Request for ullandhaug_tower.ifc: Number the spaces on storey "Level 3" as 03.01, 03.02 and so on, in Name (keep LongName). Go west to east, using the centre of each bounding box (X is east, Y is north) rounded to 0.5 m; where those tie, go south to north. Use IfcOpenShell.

First a look at what the model holds.

```python
import ifcopenshell
import ifcopenshell.util.element
import ifcopenshell.util.placement

model = ifcopenshell.open("ullandhaug_tower.ifc")
print(model.schema)
storey = next(s for s in model.by_type("IfcBuildingStorey") if s.Name == "Level 3")
spaces = [e for e in ifcopenshell.util.element.get_decomposition(storey) if e.is_a("IfcSpace")]
for e in sorted(spaces, key=lambda e: e.id()):
    origin = ifcopenshell.util.placement.get_local_placement(e.ObjectPlacement)[:3, 3]
    print(e.id(), e.Name, e.LongName, origin.round(2) + 0.0, sep=" | ")
```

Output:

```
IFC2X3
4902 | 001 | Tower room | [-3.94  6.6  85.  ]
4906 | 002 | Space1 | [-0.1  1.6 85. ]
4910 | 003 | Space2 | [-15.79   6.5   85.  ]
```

```python
import ifcopenshell
import ifcopenshell.geom
import ifcopenshell.util.element
import ifcopenshell.util.shape

model = ifcopenshell.open("ullandhaug_tower.ifc")
settings = ifcopenshell.geom.settings()
settings.set("use-world-coords", True)


def centre(element):
    shape = ifcopenshell.geom.create_shape(settings, element)
    return ifcopenshell.util.shape.get_bbox_centroid(shape.geometry)


storey = next(s for s in model.by_type("IfcBuildingStorey") if s.Name == "Level 3")
spaces = [e for e in ifcopenshell.util.element.get_decomposition(storey) if e.is_a("IfcSpace")]

# Insertion points can sit at a corner or the storey origin, so sort by the geometry (in metres).
centres = {e: centre(e) for e in spaces}
spaces.sort(key=lambda e: (round(centres[e][0] / 0.5), centres[e][1]))

for i, e in enumerate(spaces, start=1):
    number = f"03.{i:02d}"
    e.Name = number
    print(e.id(), number)

model.write("ullandhaug_tower_v2.ifc")
```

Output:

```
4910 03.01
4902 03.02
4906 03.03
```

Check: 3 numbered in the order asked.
